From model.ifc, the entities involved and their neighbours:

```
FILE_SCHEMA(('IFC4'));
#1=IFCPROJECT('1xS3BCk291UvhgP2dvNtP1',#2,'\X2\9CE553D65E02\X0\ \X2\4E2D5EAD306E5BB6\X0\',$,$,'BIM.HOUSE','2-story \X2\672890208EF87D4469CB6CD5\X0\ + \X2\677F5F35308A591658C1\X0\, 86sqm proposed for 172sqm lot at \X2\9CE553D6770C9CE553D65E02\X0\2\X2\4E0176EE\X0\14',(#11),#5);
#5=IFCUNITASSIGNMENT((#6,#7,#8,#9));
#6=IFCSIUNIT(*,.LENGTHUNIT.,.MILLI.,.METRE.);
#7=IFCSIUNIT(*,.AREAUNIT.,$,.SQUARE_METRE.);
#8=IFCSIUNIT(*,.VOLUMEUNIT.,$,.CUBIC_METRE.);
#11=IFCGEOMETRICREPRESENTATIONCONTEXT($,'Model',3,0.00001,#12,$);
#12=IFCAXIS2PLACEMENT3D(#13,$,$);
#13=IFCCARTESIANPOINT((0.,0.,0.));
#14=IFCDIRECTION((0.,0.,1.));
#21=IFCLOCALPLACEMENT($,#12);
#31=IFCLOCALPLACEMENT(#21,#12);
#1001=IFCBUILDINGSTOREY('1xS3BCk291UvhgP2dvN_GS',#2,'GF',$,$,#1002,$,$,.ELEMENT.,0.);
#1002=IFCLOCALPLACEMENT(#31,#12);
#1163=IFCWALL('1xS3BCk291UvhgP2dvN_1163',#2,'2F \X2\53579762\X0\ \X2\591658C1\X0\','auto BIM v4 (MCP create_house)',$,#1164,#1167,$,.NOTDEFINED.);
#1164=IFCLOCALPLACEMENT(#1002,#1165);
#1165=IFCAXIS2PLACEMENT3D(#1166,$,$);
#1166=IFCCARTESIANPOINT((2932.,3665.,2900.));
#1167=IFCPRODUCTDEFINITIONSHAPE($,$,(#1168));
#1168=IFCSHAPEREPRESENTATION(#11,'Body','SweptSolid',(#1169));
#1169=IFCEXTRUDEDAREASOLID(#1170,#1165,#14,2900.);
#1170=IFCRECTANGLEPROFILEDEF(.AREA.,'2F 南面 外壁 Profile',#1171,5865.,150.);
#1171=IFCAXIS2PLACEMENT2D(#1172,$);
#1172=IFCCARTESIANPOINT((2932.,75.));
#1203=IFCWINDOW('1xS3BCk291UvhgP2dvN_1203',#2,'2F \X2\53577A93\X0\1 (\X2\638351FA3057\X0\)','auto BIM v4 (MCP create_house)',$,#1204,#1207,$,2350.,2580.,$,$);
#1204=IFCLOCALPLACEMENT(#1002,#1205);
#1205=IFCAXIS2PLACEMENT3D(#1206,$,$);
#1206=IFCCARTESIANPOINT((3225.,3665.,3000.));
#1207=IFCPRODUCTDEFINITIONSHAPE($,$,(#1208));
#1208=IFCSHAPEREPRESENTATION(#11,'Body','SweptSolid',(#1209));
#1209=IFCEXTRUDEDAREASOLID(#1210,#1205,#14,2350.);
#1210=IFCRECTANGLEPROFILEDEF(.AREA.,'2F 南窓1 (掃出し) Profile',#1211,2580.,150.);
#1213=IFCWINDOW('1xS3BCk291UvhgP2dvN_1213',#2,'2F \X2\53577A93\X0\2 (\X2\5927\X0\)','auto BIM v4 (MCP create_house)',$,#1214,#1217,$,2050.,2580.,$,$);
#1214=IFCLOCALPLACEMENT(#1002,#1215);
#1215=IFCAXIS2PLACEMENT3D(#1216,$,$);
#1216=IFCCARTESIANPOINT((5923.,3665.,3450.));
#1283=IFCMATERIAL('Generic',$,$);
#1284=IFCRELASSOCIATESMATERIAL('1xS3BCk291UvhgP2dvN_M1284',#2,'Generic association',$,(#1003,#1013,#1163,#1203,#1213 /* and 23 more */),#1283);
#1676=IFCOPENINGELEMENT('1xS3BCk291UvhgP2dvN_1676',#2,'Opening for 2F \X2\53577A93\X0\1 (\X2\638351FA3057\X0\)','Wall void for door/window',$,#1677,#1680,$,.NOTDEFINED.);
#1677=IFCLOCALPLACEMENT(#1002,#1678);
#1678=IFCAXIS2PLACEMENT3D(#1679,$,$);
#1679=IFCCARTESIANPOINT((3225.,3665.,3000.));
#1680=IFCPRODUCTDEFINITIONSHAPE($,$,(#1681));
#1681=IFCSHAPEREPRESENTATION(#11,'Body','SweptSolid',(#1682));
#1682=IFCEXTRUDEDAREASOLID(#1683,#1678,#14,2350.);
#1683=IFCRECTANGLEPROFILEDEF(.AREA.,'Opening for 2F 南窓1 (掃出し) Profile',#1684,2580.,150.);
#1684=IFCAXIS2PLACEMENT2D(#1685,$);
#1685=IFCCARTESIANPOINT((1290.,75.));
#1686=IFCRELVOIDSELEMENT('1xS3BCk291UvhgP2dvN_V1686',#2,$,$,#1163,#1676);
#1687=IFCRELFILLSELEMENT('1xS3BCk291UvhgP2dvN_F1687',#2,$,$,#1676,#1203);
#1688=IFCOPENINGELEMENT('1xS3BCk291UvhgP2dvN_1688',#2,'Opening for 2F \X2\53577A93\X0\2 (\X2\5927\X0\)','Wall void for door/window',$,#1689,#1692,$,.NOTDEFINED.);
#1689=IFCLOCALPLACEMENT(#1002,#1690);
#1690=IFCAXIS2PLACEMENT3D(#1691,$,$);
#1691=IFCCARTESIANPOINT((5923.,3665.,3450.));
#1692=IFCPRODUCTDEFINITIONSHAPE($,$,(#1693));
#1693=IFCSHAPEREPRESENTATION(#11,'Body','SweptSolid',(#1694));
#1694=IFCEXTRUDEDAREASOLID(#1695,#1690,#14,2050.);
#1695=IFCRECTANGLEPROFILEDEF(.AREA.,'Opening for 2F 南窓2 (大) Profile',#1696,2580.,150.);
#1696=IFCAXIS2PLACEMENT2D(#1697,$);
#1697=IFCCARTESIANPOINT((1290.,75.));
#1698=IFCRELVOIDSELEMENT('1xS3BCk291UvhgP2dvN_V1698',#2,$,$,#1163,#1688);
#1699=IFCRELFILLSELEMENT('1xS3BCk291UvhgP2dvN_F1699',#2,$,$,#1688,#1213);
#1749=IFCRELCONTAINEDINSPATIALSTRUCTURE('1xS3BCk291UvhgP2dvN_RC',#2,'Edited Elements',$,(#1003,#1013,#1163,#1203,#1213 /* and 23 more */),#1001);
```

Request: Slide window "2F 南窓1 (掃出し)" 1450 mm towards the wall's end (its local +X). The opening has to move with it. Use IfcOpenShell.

```python
import ifcopenshell
import ifcopenshell.api.geometry
import ifcopenshell.util.placement
import ifcopenshell.util.unit

model = ifcopenshell.open("model.ifc")
unit_scale = ifcopenshell.util.unit.calculate_unit_scale(model)

window = model.by_guid("1xS3BCk291UvhgP2dvN_1203")
opening = window.FillsVoids[0].RelatingOpeningElement
wall = opening.VoidsElements[0].RelatingBuildingElement

wall_matrix = ifcopenshell.util.placement.get_local_placement(wall.ObjectPlacement)
shift = wall_matrix[:3, 0] * 1.45 / unit_scale
before = ifcopenshell.util.placement.get_local_placement(window.ObjectPlacement)[:3, 3].copy()

# The window is not placed relative to its opening, so move both.
for product in (opening, window):
    matrix = ifcopenshell.util.placement.get_local_placement(product.ObjectPlacement)
    matrix[:3, 3] += shift
    ifcopenshell.api.geometry.edit_object_placement(model, product=product, matrix=matrix, is_si=False)

after = ifcopenshell.util.placement.get_local_placement(window.ObjectPlacement)[:3, 3]
print("window moved by", (after - before).round(3) + 0.0)

model.write("model-out.ifc")
```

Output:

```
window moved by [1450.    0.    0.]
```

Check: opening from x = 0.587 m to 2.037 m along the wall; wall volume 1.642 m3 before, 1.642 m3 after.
